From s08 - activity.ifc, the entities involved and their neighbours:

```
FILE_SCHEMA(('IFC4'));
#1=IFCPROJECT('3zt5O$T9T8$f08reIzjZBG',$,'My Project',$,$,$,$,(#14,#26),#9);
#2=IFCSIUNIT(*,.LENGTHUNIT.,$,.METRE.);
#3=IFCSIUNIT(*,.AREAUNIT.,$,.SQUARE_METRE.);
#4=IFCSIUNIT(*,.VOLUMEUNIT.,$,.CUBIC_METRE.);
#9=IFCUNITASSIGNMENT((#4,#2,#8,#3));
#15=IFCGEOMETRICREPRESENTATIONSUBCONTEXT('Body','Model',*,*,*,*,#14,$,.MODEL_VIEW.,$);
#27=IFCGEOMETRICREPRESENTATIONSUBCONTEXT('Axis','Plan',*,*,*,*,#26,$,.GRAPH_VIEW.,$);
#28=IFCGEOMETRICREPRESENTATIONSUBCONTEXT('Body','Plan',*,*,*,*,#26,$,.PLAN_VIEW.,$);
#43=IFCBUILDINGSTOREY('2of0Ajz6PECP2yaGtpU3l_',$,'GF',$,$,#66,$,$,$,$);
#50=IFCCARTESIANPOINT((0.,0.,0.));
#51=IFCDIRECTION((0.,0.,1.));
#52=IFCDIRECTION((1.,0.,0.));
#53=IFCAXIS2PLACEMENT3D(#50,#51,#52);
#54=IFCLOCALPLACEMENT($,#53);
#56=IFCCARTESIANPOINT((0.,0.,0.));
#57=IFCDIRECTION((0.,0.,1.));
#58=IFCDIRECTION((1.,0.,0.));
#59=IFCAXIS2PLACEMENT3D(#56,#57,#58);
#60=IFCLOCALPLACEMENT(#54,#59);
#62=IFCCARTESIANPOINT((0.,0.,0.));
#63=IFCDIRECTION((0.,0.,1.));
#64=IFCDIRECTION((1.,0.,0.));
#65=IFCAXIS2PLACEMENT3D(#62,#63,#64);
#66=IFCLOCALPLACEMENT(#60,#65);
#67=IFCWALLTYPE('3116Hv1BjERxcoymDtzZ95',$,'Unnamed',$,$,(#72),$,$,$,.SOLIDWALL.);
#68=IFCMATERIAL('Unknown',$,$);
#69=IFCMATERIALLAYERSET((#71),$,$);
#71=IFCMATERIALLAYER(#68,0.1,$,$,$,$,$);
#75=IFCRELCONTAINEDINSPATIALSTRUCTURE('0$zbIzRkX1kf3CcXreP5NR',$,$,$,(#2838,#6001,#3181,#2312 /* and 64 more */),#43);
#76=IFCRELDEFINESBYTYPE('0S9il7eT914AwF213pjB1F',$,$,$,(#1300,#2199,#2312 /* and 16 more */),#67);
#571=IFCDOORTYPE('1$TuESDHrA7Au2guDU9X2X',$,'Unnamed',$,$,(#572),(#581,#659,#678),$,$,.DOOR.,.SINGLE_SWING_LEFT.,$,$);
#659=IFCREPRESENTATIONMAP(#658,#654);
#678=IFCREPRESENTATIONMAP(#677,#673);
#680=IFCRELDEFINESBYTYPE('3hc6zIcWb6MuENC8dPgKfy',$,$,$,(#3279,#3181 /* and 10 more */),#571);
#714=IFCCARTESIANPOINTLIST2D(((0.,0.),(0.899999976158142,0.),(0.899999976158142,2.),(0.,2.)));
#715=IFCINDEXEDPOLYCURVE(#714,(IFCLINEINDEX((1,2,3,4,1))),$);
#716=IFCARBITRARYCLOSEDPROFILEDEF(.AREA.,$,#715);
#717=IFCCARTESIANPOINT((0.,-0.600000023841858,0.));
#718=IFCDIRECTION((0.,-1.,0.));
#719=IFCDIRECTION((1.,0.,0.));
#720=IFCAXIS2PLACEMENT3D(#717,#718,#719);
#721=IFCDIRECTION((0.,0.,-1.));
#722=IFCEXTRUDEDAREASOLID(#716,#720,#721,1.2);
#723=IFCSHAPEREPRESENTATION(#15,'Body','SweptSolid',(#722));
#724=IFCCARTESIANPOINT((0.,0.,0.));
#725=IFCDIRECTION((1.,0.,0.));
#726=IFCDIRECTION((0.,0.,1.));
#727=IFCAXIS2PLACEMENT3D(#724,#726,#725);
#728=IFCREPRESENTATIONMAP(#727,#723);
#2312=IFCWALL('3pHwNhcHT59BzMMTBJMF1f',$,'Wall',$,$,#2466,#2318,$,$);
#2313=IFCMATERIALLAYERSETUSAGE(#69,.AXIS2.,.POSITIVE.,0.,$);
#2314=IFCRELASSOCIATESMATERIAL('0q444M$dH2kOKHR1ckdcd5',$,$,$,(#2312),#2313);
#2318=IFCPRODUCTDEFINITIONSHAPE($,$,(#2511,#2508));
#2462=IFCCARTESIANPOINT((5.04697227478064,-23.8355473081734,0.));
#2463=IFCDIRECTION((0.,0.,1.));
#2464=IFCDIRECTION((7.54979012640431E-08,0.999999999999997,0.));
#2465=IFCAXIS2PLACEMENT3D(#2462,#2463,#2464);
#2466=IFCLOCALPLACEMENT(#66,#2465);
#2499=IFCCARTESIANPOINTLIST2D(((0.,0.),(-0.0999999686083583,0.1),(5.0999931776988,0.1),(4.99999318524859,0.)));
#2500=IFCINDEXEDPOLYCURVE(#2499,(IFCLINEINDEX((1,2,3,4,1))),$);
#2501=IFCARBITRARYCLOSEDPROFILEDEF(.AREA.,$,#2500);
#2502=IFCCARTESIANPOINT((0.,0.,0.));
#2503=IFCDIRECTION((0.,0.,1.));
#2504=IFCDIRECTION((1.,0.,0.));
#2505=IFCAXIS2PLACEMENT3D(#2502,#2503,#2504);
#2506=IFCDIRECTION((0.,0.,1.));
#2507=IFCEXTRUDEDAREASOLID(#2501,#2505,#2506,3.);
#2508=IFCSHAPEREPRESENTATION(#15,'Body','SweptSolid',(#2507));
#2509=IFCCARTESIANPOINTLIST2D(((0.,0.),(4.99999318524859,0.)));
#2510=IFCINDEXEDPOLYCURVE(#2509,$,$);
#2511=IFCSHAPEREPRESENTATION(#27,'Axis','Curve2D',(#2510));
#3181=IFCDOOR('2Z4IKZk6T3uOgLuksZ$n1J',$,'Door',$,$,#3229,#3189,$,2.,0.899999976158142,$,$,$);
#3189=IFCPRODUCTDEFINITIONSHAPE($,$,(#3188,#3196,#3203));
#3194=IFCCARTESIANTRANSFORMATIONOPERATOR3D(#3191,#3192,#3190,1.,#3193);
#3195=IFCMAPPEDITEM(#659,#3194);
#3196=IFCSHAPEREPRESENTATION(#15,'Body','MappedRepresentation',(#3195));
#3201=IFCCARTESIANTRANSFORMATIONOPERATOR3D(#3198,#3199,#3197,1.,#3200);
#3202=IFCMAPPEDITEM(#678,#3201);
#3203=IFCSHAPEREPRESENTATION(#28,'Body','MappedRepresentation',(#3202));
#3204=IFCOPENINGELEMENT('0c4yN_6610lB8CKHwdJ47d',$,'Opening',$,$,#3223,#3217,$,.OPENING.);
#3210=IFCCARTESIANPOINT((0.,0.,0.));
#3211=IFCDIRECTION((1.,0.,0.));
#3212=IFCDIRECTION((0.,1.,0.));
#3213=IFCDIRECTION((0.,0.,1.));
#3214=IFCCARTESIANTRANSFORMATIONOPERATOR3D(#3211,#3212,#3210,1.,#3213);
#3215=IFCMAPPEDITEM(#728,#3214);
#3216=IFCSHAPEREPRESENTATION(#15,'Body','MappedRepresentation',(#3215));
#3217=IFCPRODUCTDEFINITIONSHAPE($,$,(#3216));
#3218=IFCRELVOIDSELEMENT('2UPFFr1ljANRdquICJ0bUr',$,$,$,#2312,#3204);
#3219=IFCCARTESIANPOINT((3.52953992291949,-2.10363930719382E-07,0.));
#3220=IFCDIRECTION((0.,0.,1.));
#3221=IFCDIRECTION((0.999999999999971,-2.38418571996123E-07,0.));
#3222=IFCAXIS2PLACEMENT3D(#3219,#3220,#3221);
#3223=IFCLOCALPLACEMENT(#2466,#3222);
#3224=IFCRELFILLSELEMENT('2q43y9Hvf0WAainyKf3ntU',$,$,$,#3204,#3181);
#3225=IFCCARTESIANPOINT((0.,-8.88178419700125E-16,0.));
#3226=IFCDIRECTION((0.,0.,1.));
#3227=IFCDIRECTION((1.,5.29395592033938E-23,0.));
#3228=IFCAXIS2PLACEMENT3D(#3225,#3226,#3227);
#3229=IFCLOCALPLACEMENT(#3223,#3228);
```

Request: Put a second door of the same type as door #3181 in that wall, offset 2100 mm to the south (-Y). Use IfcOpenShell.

```python
import ifcopenshell
import ifcopenshell.api.feature
import ifcopenshell.api.geometry
import ifcopenshell.api.root
import ifcopenshell.geom
import ifcopenshell.util.element
import ifcopenshell.util.placement
import ifcopenshell.util.shape
import ifcopenshell.util.unit

model = ifcopenshell.open("s08 - activity.ifc")
unit_scale = ifcopenshell.util.unit.calculate_unit_scale(model)
settings = ifcopenshell.geom.settings()


def volume(element):
    """Net volume in cubic metres, openings subtracted."""
    shape = ifcopenshell.geom.create_shape(settings, element)
    return ifcopenshell.util.shape.get_volume(shape.geometry)


door = model.by_guid("2Z4IKZk6T3uOgLuksZ$n1J")
opening = door.FillsVoids[0].RelatingOpeningElement
wall = opening.VoidsElements[0].RelatingBuildingElement
before = volume(wall)
shift = ifcopenshell.util.placement.get_local_placement(wall.ObjectPlacement)[:3, 0] * -2.1 / unit_scale

# copy_class copies the void relationship, type, container and properties, but no geometry.
new_opening = ifcopenshell.api.root.copy_class(model, product=opening)
new_opening.Representation = ifcopenshell.util.element.copy_deep(
    model, opening.Representation, exclude=["IfcGeometricRepresentationContext", "IfcRepresentationMap"]
)
new_door = ifcopenshell.api.root.copy_class(model, product=door)
new_door.Representation = ifcopenshell.util.element.copy_deep(
    model, door.Representation, exclude=["IfcGeometricRepresentationContext", "IfcRepresentationMap"]
)
ifcopenshell.api.feature.add_filling(model, opening=new_opening, element=new_door)

for old, new in ((opening, new_opening), (door, new_door)):
    matrix = ifcopenshell.util.placement.get_local_placement(old.ObjectPlacement)
    matrix[:3, 3] += shift
    ifcopenshell.api.geometry.edit_object_placement(model, product=new, matrix=matrix, is_si=False)

after = volume(wall)

print(f"wall volume {before:.3f} -> {after:.3f} m3")

model.write("s08 - activity_rev.ifc")
```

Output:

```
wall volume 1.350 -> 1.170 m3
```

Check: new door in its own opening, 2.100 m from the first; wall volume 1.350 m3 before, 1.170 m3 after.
